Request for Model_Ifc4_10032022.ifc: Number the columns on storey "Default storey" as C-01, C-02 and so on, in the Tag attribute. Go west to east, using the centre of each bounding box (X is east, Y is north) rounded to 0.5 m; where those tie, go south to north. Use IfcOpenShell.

First a look at what the model holds.

```python
import ifcopenshell
import ifcopenshell.util.element
import ifcopenshell.util.placement

model = ifcopenshell.open("Model_Ifc4_10032022.ifc")
print(model.schema)
storey = next(s for s in model.by_type("IfcBuildingStorey") if s.Name == "Default storey")
columns = [e for e in ifcopenshell.util.element.get_decomposition(storey) if e.is_a("IfcColumn")]
for e in sorted(columns, key=lambda e: e.id()):
    origin = ifcopenshell.util.placement.get_local_placement(e.ObjectPlacement)[:3, 3]
    print(e.id(), e.Tag, e.Name, origin.round(2) + 0.0, sep=" | ")
```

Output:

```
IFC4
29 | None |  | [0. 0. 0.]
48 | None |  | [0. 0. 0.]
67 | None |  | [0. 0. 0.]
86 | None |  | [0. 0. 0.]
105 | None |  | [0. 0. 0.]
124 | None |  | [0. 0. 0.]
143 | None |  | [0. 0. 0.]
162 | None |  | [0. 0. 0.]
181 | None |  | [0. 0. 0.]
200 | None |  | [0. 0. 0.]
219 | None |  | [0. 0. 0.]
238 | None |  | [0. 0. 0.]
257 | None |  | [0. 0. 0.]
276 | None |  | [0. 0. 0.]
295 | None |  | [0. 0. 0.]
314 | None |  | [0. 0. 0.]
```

```python
import ifcopenshell
import ifcopenshell.geom
import ifcopenshell.util.element
import ifcopenshell.util.shape

model = ifcopenshell.open("Model_Ifc4_10032022.ifc")
settings = ifcopenshell.geom.settings()
settings.set("use-world-coords", True)


def centre(element):
    shape = ifcopenshell.geom.create_shape(settings, element)
    return ifcopenshell.util.shape.get_bbox_centroid(shape.geometry)


storey = next(s for s in model.by_type("IfcBuildingStorey") if s.Name == "Default storey")
columns = [e for e in ifcopenshell.util.element.get_decomposition(storey) if e.is_a("IfcColumn")]

# Insertion points can sit at a corner or the storey origin, so sort by the geometry (in metres).
centres = {e: centre(e) for e in columns}
columns.sort(key=lambda e: (round(centres[e][0] / 0.5), centres[e][1]))

for i, e in enumerate(columns, start=1):
    number = f"C-{i:02d}"
    e.Tag = number
    print(e.id(), number)

model.write("Model_Ifc4_10032022_edited.ifc")
```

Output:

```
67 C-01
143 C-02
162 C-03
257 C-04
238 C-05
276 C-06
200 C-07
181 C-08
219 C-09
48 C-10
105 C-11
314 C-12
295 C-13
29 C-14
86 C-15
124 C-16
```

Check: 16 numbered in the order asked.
